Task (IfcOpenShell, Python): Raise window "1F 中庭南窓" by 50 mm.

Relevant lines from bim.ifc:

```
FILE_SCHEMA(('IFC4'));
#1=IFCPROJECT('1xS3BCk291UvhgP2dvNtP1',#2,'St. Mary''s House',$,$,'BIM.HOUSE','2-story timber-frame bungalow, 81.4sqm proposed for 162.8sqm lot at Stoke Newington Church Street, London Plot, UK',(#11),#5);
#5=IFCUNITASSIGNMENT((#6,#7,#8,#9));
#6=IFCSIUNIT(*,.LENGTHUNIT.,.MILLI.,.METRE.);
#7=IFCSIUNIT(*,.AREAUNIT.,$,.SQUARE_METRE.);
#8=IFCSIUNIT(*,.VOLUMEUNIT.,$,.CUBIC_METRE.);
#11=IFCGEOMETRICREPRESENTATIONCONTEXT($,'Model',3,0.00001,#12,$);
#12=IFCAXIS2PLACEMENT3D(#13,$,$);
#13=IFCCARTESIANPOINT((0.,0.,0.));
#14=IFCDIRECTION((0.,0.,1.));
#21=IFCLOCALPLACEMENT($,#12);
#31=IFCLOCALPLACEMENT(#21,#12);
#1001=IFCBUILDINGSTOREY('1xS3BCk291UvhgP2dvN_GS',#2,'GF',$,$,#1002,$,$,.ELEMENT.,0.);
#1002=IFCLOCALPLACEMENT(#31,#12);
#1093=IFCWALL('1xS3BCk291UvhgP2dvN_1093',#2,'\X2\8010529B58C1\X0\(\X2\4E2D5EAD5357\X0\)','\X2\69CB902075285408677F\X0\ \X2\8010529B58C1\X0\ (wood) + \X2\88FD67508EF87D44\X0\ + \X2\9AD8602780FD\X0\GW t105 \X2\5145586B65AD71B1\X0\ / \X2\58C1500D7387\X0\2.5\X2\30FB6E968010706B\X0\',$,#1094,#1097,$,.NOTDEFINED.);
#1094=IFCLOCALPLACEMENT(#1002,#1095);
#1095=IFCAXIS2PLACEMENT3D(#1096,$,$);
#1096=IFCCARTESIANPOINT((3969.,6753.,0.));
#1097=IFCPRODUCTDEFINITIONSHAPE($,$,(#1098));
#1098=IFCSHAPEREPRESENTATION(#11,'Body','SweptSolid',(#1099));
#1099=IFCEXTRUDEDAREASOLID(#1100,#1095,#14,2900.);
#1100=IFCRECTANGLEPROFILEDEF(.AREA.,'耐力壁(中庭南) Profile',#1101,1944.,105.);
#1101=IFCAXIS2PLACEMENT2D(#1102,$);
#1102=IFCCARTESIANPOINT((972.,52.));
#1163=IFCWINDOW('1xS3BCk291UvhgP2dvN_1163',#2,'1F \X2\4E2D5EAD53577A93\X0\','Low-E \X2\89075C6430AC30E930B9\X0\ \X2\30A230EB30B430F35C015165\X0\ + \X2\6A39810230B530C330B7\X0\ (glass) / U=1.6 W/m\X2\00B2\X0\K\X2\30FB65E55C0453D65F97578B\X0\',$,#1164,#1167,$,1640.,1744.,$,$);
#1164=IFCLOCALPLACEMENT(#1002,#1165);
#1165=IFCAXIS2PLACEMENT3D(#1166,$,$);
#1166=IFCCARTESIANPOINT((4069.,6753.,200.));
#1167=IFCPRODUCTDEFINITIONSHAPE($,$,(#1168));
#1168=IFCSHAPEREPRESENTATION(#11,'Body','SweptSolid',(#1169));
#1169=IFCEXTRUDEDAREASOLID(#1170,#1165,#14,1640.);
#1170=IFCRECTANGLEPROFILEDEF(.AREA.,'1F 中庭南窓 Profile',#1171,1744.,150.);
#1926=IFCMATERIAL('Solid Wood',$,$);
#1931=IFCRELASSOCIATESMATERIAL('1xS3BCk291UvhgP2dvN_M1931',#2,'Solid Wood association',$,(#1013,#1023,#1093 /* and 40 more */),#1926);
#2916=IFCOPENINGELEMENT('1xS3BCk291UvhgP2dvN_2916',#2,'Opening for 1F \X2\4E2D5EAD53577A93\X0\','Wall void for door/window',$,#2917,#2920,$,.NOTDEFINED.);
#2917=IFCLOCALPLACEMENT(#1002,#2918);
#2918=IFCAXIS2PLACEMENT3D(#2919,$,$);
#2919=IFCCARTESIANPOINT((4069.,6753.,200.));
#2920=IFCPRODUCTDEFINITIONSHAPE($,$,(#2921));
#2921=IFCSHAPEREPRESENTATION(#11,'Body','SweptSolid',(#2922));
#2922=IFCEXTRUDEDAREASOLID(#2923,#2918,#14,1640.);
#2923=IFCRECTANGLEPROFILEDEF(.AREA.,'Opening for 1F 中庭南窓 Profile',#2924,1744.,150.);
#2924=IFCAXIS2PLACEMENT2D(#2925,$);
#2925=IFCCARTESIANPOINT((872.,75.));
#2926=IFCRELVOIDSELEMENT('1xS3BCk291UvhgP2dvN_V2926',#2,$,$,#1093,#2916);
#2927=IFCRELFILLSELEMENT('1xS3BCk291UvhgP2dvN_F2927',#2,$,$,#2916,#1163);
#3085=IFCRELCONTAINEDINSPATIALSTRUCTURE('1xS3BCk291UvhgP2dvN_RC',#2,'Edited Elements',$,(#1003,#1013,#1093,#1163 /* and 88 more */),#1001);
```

```python
import numpy as np
import ifcopenshell
import ifcopenshell.api.geometry
import ifcopenshell.util.placement
import ifcopenshell.util.unit

model = ifcopenshell.open("bim.ifc")
unit_scale = ifcopenshell.util.unit.calculate_unit_scale(model)

window = model.by_guid("1xS3BCk291UvhgP2dvN_1163")
opening = window.FillsVoids[0].RelatingOpeningElement
dz = 0.05 / unit_scale

shift = np.array([0.0, 0.0, dz])
# The window is not placed relative to its opening, so move both.
for product in (opening, window):
    matrix = ifcopenshell.util.placement.get_local_placement(product.ObjectPlacement)
    matrix[:3, 3] += shift
    ifcopenshell.api.geometry.edit_object_placement(model, product=product, matrix=matrix, is_si=False)

print(f"moved by {dz * unit_scale:+.3f} m")

model.write("bim_updated.ifc")
```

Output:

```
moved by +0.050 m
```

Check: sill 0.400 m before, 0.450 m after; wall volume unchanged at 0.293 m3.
